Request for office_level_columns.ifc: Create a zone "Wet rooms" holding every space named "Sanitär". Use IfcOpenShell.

First a look at what the model holds.

```python
import ifcopenshell

model = ifcopenshell.open("office_level_columns.ifc")
print(model.schema)
seen = {}
for space in model.by_type("IfcSpace"):
    seen[space.LongName] = seen.get(space.LongName, 0) + 1
for name, count in sorted(seen.items(), key=str):
    print(count, "x", name)
print("zones:", [z.Name for z in model.by_type("IfcZone")][:20])
```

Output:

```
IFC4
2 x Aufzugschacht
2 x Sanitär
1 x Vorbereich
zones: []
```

```python
import ifcopenshell
import ifcopenshell.api.group
import ifcopenshell.api.root

model = ifcopenshell.open("office_level_columns.ifc")

names = {"Sanitär"}
spaces = [s for s in model.by_type("IfcSpace") if s.LongName in names]

zone = ifcopenshell.api.root.create_entity(model, ifc_class="IfcZone", name="Wet rooms")
ifcopenshell.api.group.assign_group(model, products=spaces, group=zone)
print(len(spaces), "spaces in", zone.Name)

model.write("office_level_columns_v2.ifc")
```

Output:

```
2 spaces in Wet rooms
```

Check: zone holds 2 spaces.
